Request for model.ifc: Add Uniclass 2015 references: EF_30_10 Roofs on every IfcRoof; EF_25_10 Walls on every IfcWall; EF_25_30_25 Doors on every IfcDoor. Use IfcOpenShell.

First a look at what the model holds.

```python
import ifcopenshell

model = ifcopenshell.open("model.ifc")
print(model.schema)
print("classifications:", [c.Name for c in model.by_type("IfcClassification")])
for ifc_class in ("IfcDoor", "IfcRoof", "IfcStair", "IfcWall", "IfcWindow"):
    print(ifc_class, len(model.by_type(ifc_class)))
```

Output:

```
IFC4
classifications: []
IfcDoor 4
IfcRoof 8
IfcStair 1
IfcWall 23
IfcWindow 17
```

```python
import ifcopenshell
import ifcopenshell.api.classification

model = ifcopenshell.open("model.ifc")

system = ifcopenshell.api.classification.add_classification(model, classification="Uniclass 2015")

codes = {
    "IfcRoof": ("EF_30_10", "Roofs"),
    "IfcWall": ("EF_25_10", "Walls"),
    "IfcDoor": ("EF_25_30_25", "Doors"),
}
for ifc_class, (code, name) in codes.items():
    products = model.by_type(ifc_class)
    ifcopenshell.api.classification.add_reference(
        model, products=products, classification=system, identification=code, name=name
    )
    print(code, len(products))

model.write("model_edited.ifc")
```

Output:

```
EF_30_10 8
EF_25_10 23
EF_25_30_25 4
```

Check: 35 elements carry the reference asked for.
